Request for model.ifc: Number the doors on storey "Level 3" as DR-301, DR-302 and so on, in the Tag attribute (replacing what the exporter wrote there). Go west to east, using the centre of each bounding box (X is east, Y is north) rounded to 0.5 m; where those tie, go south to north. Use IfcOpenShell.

First a look at what the model holds.

```python
import ifcopenshell
import ifcopenshell.util.element
import ifcopenshell.util.placement

model = ifcopenshell.open("model.ifc")
print(model.schema)
storey = next(s for s in model.by_type("IfcBuildingStorey") if s.Name == "Level 3")
doors = [e for e in ifcopenshell.util.element.get_decomposition(storey) if e.is_a("IfcDoor")]
for e in sorted(doors, key=lambda e: e.id()):
    origin = ifcopenshell.util.placement.get_local_placement(e.ObjectPlacement)[:3, 3]
    print(e.id(), e.Tag, e.Name, origin.round(2) + 0.0, sep=" | ")
```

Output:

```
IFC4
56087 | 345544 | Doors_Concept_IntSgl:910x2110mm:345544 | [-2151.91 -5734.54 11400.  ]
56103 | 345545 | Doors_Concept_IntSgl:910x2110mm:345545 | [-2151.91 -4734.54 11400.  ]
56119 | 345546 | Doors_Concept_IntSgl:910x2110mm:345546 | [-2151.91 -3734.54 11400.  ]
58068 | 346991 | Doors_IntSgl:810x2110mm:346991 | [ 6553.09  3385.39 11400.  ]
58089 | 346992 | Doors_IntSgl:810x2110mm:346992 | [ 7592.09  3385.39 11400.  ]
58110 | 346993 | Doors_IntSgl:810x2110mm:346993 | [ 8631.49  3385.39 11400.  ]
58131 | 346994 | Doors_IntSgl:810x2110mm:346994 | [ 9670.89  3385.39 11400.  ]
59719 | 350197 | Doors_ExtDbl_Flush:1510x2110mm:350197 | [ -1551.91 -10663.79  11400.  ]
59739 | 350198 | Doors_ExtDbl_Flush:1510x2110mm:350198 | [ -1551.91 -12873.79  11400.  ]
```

```python
import ifcopenshell
import ifcopenshell.geom
import ifcopenshell.util.element
import ifcopenshell.util.shape

model = ifcopenshell.open("model.ifc")
settings = ifcopenshell.geom.settings()
settings.set("use-world-coords", True)


def centre(element):
    shape = ifcopenshell.geom.create_shape(settings, element)
    return ifcopenshell.util.shape.get_bbox_centroid(shape.geometry)


storey = next(s for s in model.by_type("IfcBuildingStorey") if s.Name == "Level 3")
doors = [e for e in ifcopenshell.util.element.get_decomposition(storey) if e.is_a("IfcDoor")]

# Insertion points can sit at a corner or the storey origin, so sort by the geometry (in metres).
centres = {e: centre(e) for e in doors}
doors.sort(key=lambda e: (round(centres[e][0] / 0.5), centres[e][1]))

for i, e in enumerate(doors, start=1):
    number = f"DR-3{i:02d}"
    e.Tag = number
    print(e.id(), number)

model.write("model_updated.ifc")
```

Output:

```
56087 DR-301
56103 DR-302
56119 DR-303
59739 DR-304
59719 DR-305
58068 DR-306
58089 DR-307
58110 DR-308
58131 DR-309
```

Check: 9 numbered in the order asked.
